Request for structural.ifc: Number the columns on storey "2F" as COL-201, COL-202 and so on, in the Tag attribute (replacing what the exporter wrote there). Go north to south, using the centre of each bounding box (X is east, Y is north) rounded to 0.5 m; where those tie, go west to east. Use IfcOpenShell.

First a look at what the model holds.

```python
import ifcopenshell
import ifcopenshell.util.element
import ifcopenshell.util.placement

model = ifcopenshell.open("structural.ifc")
print(model.schema)
storey = next(s for s in model.by_type("IfcBuildingStorey") if s.Name == "2F")
columns = [e for e in ifcopenshell.util.element.get_decomposition(storey) if e.is_a("IfcColumn")]
for e in sorted(columns, key=lambda e: e.id()):
    origin = ifcopenshell.util.placement.get_local_placement(e.ObjectPlacement)[:3, 3]
    print(e.id(), e.Tag, e.Name, origin.round(2) + 0.0, sep=" | ")
```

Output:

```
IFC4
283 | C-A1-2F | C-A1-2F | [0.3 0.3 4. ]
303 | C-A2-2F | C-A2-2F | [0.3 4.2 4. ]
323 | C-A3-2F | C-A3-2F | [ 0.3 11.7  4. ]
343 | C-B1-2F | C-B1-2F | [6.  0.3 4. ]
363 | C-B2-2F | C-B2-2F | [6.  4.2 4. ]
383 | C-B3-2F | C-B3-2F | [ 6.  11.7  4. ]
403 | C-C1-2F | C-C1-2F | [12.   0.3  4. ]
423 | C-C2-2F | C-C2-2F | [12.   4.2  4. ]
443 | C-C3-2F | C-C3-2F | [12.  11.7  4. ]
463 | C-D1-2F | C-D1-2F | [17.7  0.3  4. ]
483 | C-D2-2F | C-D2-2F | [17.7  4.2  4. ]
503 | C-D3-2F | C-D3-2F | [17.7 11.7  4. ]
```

```python
import ifcopenshell
import ifcopenshell.geom
import ifcopenshell.util.element
import ifcopenshell.util.shape

model = ifcopenshell.open("structural.ifc")
settings = ifcopenshell.geom.settings()
settings.set("use-world-coords", True)


def centre(element):
    shape = ifcopenshell.geom.create_shape(settings, element)
    return ifcopenshell.util.shape.get_bbox_centroid(shape.geometry)


storey = next(s for s in model.by_type("IfcBuildingStorey") if s.Name == "2F")
columns = [e for e in ifcopenshell.util.element.get_decomposition(storey) if e.is_a("IfcColumn")]

# Insertion points can sit at a corner or the storey origin, so sort by the geometry (in metres).
centres = {e: centre(e) for e in columns}
columns.sort(key=lambda e: (-round(centres[e][1] / 0.5), centres[e][0]))

for i, e in enumerate(columns, start=1):
    number = f"COL-2{i:02d}"
    e.Tag = number
    print(e.id(), number)

model.write("structural_edited.ifc")
```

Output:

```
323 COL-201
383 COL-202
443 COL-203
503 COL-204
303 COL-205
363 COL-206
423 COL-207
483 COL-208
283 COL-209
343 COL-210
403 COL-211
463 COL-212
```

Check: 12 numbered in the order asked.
